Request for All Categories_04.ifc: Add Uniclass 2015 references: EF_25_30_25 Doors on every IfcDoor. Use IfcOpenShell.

First a look at what the model holds.

```python
import ifcopenshell

model = ifcopenshell.open("All Categories_04.ifc")
print(model.schema)
print("classifications:", [c.Name for c in model.by_type("IfcClassification")])
for ifc_class in ("IfcDoor", "IfcRoof", "IfcStair", "IfcWall", "IfcWindow"):
    print(ifc_class, len(model.by_type(ifc_class)))
```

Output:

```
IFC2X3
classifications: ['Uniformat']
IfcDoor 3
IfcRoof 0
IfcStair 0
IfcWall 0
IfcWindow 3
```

```python
import ifcopenshell
import ifcopenshell.api.classification

model = ifcopenshell.open("All Categories_04.ifc")

# IFC2X3 requires Source and Edition and has no link from the project to the system.
system = model.create_entity("IfcClassification", Source="NBS", Edition="2015", Name="Uniclass 2015")

codes = {
    "IfcDoor": ("EF_25_30_25", "Doors"),
}
for ifc_class, (code, name) in codes.items():
    products = model.by_type(ifc_class)
    ifcopenshell.api.classification.add_reference(
        model, products=products, classification=system, identification=code, name=name
    )
    print(code, len(products))

model.write("All Categories_04_updated.ifc")
```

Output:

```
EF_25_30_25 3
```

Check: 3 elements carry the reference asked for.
